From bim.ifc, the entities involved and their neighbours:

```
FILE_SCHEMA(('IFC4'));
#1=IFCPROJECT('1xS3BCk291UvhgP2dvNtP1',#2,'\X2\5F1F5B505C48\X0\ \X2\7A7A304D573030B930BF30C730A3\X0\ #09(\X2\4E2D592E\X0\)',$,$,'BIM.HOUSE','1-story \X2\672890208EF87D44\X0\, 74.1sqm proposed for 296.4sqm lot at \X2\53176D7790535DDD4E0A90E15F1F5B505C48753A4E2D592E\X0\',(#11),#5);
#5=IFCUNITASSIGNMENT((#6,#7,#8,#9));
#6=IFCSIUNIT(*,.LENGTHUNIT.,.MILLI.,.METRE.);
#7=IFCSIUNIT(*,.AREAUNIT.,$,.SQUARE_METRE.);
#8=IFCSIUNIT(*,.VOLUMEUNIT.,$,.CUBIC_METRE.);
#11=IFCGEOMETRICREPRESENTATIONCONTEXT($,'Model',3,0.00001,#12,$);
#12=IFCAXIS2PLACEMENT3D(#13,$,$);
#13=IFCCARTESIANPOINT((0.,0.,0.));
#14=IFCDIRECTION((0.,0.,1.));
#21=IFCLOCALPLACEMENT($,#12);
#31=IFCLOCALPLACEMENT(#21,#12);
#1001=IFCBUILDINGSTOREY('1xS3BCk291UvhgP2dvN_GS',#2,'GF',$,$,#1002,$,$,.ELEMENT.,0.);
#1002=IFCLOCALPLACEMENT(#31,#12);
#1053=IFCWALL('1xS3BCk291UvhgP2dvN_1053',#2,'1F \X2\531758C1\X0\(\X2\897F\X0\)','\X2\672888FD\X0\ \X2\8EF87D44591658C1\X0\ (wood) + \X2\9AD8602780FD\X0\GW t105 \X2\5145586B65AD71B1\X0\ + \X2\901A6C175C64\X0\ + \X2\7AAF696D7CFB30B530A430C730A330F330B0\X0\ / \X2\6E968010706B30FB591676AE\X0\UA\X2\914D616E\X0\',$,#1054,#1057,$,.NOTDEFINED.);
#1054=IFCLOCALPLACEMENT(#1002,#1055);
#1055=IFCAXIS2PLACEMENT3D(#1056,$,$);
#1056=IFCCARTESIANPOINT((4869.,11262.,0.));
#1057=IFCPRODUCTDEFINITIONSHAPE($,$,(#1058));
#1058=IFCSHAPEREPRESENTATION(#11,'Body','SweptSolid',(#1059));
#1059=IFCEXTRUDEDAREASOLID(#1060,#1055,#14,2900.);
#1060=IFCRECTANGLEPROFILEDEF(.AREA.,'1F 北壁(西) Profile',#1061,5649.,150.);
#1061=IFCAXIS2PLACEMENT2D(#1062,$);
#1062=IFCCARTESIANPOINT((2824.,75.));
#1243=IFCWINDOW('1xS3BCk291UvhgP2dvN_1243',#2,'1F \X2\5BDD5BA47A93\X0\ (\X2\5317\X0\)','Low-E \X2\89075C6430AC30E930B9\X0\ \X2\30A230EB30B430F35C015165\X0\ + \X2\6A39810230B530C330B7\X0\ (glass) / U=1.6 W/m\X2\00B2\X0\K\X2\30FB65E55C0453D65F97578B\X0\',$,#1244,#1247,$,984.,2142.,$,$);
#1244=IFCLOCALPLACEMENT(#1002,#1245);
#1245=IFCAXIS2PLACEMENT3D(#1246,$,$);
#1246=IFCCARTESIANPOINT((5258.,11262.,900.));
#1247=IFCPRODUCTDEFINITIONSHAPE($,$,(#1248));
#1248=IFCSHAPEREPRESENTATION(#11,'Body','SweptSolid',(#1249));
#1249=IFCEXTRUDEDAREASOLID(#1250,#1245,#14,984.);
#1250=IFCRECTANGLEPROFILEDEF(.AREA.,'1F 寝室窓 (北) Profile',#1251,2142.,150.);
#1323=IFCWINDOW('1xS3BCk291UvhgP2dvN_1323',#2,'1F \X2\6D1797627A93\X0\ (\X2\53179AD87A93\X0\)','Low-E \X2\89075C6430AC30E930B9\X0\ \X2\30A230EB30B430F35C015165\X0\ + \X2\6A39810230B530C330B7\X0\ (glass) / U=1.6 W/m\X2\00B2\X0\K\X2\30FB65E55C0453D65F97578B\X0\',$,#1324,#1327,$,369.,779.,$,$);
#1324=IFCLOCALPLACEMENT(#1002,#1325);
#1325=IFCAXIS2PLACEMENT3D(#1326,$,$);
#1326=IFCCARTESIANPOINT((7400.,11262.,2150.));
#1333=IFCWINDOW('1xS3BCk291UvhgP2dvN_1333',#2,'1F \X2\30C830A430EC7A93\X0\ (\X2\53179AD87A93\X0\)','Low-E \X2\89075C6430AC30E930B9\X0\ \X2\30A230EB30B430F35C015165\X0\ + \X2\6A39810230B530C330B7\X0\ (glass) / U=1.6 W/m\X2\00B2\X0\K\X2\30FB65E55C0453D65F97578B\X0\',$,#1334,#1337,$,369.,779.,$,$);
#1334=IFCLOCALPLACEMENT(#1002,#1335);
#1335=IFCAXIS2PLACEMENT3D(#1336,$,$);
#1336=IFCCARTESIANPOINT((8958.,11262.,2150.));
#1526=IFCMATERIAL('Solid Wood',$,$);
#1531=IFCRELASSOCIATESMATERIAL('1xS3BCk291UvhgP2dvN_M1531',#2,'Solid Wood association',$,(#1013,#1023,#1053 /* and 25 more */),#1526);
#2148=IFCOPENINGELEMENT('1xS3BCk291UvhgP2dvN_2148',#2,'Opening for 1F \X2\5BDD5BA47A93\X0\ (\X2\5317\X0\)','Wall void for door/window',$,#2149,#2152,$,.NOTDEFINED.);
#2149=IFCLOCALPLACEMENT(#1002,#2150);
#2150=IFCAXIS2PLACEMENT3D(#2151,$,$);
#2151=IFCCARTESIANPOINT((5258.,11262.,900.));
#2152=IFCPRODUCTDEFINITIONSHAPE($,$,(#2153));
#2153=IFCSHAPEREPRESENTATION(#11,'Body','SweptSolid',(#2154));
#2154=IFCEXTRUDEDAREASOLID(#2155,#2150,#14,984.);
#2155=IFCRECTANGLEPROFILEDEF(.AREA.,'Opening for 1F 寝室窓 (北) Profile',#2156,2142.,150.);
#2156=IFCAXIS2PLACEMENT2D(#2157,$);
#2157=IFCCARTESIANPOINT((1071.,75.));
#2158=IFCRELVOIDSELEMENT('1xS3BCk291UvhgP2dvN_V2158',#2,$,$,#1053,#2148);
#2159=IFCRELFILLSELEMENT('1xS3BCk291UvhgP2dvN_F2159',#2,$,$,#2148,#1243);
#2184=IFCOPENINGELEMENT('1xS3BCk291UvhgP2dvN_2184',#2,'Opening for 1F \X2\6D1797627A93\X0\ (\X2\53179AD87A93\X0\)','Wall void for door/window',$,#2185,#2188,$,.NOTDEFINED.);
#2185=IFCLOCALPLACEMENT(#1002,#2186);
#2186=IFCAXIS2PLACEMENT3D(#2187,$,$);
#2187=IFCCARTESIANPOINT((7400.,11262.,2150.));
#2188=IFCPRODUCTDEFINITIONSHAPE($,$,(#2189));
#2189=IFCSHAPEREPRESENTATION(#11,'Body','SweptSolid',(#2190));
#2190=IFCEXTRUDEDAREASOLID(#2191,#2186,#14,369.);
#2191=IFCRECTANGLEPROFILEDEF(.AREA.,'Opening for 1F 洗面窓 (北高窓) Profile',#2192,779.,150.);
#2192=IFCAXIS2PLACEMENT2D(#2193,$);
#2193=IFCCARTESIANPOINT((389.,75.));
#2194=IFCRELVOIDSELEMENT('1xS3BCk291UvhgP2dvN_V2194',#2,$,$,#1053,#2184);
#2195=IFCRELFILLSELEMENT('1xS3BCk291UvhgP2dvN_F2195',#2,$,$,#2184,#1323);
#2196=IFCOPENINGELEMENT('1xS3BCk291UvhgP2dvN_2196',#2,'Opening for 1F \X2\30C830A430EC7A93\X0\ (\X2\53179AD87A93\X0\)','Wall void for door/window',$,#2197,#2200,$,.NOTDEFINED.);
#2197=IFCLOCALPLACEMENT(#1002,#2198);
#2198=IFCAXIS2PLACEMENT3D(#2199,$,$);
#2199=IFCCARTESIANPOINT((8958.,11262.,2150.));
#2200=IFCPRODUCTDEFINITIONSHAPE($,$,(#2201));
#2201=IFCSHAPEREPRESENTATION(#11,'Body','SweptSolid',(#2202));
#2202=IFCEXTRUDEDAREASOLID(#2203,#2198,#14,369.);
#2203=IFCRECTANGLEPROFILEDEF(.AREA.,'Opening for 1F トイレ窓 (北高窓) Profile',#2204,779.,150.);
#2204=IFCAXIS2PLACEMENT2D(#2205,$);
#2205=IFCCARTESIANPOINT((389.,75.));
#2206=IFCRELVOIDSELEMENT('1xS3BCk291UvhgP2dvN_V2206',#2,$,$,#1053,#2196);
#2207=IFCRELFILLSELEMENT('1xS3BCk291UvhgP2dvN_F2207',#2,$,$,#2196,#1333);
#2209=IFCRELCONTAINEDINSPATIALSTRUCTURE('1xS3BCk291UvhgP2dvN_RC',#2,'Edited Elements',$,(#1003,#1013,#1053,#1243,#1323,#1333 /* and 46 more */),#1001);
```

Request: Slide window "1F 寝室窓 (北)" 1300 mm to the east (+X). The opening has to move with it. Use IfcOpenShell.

```python
import ifcopenshell
import ifcopenshell.api.geometry
import ifcopenshell.util.placement
import ifcopenshell.util.unit

model = ifcopenshell.open("bim.ifc")
unit_scale = ifcopenshell.util.unit.calculate_unit_scale(model)

window = model.by_guid("1xS3BCk291UvhgP2dvN_1243")
opening = window.FillsVoids[0].RelatingOpeningElement
wall = opening.VoidsElements[0].RelatingBuildingElement

wall_matrix = ifcopenshell.util.placement.get_local_placement(wall.ObjectPlacement)
shift = wall_matrix[:3, 0] * 1.3 / unit_scale
before = ifcopenshell.util.placement.get_local_placement(window.ObjectPlacement)[:3, 3].copy()

# The window is not placed relative to its opening, so move both.
for product in (opening, window):
    matrix = ifcopenshell.util.placement.get_local_placement(product.ObjectPlacement)
    matrix[:3, 3] += shift
    ifcopenshell.api.geometry.edit_object_placement(model, product=product, matrix=matrix, is_si=False)

after = ifcopenshell.util.placement.get_local_placement(window.ObjectPlacement)[:3, 3]
print("window moved by", (after - before).round(3) + 0.0)

model.write("bim-out.ifc")
```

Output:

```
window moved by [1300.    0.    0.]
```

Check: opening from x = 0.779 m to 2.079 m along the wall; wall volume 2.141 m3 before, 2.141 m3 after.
